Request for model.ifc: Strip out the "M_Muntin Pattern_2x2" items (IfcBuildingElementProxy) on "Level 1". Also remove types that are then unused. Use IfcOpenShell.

First a look at what the model holds.

```python
import ifcopenshell
import ifcopenshell.util.element

model = ifcopenshell.open("model.ifc")
print(model.schema)
storey = next(s for s in model.by_type("IfcBuildingStorey") if s.Name == "Level 1")
proxies = [e for e in ifcopenshell.util.element.get_decomposition(storey) if e.is_a("IfcBuildingElementProxy")]
seen = {}
for e in proxies:
    element_type = ifcopenshell.util.element.get_type(e)
    name = element_type.Name if element_type not in (None, e) else None
    seen[name] = seen.get(name, 0) + 1
for name, count in sorted(seen.items(), key=str):
    print(count, "x", name)
```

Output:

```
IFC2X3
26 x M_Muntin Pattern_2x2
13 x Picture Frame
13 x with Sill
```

```python
import ifcopenshell
import ifcopenshell.api.root
import ifcopenshell.util.element

model = ifcopenshell.open("model.ifc")

storey = next(s for s in model.by_type("IfcBuildingStorey") if s.Name == "Level 1")
proxies = [e for e in ifcopenshell.util.element.get_decomposition(storey) if e.is_a("IfcBuildingElementProxy")]
targets = [e for e in proxies if (t := ifcopenshell.util.element.get_type(e)) not in (None, e) and t.Name == "M_Muntin Pattern_2x2"]
types = {ifcopenshell.util.element.get_type(e) for e in targets} - {None, *targets}

for e in targets:
    ifcopenshell.api.root.remove_product(model, product=e)
print(len(targets), "removed")

unused = [t for t in types if not ifcopenshell.util.element.get_types(t)]
for t in unused:
    ifcopenshell.api.root.remove_product(model, product=t)
print(len(unused), "unused types removed")

model.write("model-out.ifc")
```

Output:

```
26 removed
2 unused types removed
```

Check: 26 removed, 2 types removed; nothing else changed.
